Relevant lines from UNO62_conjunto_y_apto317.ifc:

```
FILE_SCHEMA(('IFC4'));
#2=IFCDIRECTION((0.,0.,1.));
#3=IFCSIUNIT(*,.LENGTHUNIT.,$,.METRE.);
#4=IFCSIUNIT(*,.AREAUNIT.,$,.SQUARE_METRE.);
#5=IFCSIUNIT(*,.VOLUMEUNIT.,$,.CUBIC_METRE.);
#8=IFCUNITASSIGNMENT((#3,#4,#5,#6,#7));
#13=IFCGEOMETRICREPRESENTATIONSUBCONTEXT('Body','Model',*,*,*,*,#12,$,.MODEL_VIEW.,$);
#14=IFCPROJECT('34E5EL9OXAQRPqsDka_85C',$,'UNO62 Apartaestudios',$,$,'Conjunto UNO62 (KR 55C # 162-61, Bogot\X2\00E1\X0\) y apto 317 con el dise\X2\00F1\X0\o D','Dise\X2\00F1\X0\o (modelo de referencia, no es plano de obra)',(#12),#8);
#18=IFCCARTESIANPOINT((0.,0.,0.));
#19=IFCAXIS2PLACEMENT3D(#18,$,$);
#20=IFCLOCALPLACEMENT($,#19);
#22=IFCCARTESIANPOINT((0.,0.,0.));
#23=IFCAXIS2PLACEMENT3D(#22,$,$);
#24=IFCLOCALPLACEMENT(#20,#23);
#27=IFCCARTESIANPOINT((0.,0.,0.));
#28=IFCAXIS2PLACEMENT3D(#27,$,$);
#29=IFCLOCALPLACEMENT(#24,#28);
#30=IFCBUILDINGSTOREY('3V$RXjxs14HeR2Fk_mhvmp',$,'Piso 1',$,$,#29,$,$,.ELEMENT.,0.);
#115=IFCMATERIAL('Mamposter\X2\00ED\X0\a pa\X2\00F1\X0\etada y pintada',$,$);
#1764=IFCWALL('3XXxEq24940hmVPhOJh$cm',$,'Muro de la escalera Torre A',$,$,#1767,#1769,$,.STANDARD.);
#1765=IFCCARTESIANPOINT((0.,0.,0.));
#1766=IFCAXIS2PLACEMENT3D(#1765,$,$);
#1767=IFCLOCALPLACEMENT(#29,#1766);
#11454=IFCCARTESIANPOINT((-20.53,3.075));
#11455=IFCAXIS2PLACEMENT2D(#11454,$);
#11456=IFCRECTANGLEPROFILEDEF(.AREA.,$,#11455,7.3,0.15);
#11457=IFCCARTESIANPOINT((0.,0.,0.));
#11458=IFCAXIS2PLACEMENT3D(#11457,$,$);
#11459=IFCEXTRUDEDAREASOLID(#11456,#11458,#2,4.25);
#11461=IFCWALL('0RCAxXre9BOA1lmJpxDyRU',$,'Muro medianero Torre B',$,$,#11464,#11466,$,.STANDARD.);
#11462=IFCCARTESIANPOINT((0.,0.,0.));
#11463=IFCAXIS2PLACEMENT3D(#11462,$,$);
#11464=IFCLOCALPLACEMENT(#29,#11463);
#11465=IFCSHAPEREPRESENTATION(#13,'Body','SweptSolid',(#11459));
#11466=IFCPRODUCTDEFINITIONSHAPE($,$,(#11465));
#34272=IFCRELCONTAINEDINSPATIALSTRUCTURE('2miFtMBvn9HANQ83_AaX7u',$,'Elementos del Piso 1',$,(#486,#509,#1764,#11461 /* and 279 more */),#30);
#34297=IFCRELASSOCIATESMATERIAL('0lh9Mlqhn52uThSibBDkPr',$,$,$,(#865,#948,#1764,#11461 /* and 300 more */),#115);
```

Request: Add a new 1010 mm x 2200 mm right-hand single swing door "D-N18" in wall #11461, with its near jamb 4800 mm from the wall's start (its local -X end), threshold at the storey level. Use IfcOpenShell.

```python
import numpy as np
import ifcopenshell
import ifcopenshell.api.feature
import ifcopenshell.api.geometry
import ifcopenshell.api.root
import ifcopenshell.api.spatial
import ifcopenshell.geom
import ifcopenshell.util.element
import ifcopenshell.util.placement
import ifcopenshell.util.representation
import ifcopenshell.util.shape
import ifcopenshell.util.unit

model = ifcopenshell.open("UNO62_conjunto_y_apto317.ifc")
unit_scale = ifcopenshell.util.unit.calculate_unit_scale(model)
settings = ifcopenshell.geom.settings()


def volume(element):
    """Net volume in cubic metres, openings subtracted."""
    shape = ifcopenshell.geom.create_shape(settings, element)
    return ifcopenshell.util.shape.get_volume(shape.geometry)


wall = model.by_id(11461)
storey = ifcopenshell.util.element.get_container(wall, ifc_class="IfcBuildingStorey")
context = ifcopenshell.util.representation.get_context(model, "Model", "Body", "MODEL_VIEW")
before = volume(wall)

width, height, from_end, sill = 1.01, 2.2, 4.8, 0.0  # metres

# The wall runs along its own X axis, and the end named is its -X end.
wall_shape = ifcopenshell.geom.create_shape(settings, wall)
x, y, z = ifcopenshell.util.shape.get_vertices(wall_shape.geometry).T
start = x.min() + from_end
face, thickness = float(y.min()), float(y.max() - y.min())
wall_matrix = ifcopenshell.util.placement.get_local_placement(wall.ObjectPlacement)
level = ifcopenshell.util.placement.get_local_placement(storey.ObjectPlacement)[2, 3]


def in_wall(x, y):
    """Placement at x, y metres in the wall's axes, at sill height."""
    matrix = wall_matrix.copy()
    matrix[:, 3] = wall_matrix @ np.array([x / unit_scale, y / unit_scale, 0.0, 1.0])
    matrix[2, 3] = level + sill / unit_scale
    return matrix


# Opening: a box that overshoots both wall faces by 50 mm.
opening = ifcopenshell.api.root.create_entity(model, ifc_class="IfcOpeningElement", predefined_type="OPENING")
box = ifcopenshell.api.geometry.add_wall_representation(
    model, context=context, length=width, height=height, thickness=thickness + 0.1
)
ifcopenshell.api.geometry.assign_representation(model, product=opening, representation=box)
ifcopenshell.api.geometry.edit_object_placement(model, product=opening, matrix=in_wall(start, face - 0.05), is_si=False)
ifcopenshell.api.feature.add_feature(model, feature=opening, element=wall)

door = ifcopenshell.api.root.create_entity(model, ifc_class="IfcDoor", name="D-N18", predefined_type="DOOR")
door.OverallWidth, door.OverallHeight = width / unit_scale, height / unit_scale
door.OperationType = "SINGLE_SWING_RIGHT"
body = ifcopenshell.api.geometry.add_door_representation(
    model,
    context=context,
    overall_width=door.OverallWidth,
    overall_height=door.OverallHeight,
    operation_type="SINGLE_SWING_RIGHT",
    lining_properties={"LiningDepth": thickness / unit_scale, "ThresholdDepth": thickness / unit_scale},
)
ifcopenshell.api.geometry.assign_representation(model, product=door, representation=body)
ifcopenshell.api.spatial.assign_container(model, products=[door], relating_structure=storey)
ifcopenshell.api.feature.add_filling(model, opening=opening, element=door)

# The lining spans the wall, so the door starts at the wall face.
ifcopenshell.api.geometry.edit_object_placement(model, product=door, matrix=in_wall(start, face), is_si=False)

after = volume(wall)

print(f"wall volume {before:.3f} -> {after:.3f} m3")

model.write("UNO62_conjunto_y_apto317-out.ifc")
```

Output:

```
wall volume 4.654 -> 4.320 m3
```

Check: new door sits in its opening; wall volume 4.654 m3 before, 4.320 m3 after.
